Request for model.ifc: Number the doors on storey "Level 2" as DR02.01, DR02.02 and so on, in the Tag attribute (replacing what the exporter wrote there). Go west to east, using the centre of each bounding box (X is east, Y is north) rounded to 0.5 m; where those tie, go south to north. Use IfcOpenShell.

First a look at what the model holds.

```python
import ifcopenshell
import ifcopenshell.util.element
import ifcopenshell.util.placement

model = ifcopenshell.open("model.ifc")
print(model.schema)
storey = next(s for s in model.by_type("IfcBuildingStorey") if s.Name == "Level 2")
doors = [e for e in ifcopenshell.util.element.get_decomposition(storey) if e.is_a("IfcDoor")]
for e in sorted(doors, key=lambda e: e.id()):
    origin = ifcopenshell.util.placement.get_local_placement(e.ObjectPlacement)[:3, 3]
    print(e.id(), e.Tag, e.Name, origin.round(2) + 0.0, sep=" | ")
```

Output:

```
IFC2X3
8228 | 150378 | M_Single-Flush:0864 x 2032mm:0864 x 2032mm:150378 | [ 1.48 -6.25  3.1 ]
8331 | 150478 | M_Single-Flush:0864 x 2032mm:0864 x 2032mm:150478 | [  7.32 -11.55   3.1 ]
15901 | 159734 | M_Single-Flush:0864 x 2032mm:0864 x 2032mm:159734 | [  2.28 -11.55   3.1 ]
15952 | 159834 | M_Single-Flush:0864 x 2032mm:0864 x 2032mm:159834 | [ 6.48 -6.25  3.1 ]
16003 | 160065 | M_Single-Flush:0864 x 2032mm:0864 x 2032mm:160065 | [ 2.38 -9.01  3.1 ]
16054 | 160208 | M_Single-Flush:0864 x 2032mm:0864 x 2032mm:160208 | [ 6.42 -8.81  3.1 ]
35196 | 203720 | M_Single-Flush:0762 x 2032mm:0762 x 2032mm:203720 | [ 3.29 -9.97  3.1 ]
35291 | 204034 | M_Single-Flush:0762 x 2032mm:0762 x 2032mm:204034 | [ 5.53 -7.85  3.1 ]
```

```python
import ifcopenshell
import ifcopenshell.geom
import ifcopenshell.util.element
import ifcopenshell.util.shape

model = ifcopenshell.open("model.ifc")
settings = ifcopenshell.geom.settings()
settings.set("use-world-coords", True)


def centre(element):
    shape = ifcopenshell.geom.create_shape(settings, element)
    return ifcopenshell.util.shape.get_bbox_centroid(shape.geometry)


storey = next(s for s in model.by_type("IfcBuildingStorey") if s.Name == "Level 2")
doors = [e for e in ifcopenshell.util.element.get_decomposition(storey) if e.is_a("IfcDoor")]

# Insertion points can sit at a corner or the storey origin, so sort by the geometry (in metres).
centres = {e: centre(e) for e in doors}
doors.sort(key=lambda e: (round(centres[e][0] / 0.5), centres[e][1]))

for i, e in enumerate(doors, start=1):
    number = f"DR02.{i:02d}"
    e.Tag = number
    print(e.id(), number)

model.write("model_rev.ifc")
```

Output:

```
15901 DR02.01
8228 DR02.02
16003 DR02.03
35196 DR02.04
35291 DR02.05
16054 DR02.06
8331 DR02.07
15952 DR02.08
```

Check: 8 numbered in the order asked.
